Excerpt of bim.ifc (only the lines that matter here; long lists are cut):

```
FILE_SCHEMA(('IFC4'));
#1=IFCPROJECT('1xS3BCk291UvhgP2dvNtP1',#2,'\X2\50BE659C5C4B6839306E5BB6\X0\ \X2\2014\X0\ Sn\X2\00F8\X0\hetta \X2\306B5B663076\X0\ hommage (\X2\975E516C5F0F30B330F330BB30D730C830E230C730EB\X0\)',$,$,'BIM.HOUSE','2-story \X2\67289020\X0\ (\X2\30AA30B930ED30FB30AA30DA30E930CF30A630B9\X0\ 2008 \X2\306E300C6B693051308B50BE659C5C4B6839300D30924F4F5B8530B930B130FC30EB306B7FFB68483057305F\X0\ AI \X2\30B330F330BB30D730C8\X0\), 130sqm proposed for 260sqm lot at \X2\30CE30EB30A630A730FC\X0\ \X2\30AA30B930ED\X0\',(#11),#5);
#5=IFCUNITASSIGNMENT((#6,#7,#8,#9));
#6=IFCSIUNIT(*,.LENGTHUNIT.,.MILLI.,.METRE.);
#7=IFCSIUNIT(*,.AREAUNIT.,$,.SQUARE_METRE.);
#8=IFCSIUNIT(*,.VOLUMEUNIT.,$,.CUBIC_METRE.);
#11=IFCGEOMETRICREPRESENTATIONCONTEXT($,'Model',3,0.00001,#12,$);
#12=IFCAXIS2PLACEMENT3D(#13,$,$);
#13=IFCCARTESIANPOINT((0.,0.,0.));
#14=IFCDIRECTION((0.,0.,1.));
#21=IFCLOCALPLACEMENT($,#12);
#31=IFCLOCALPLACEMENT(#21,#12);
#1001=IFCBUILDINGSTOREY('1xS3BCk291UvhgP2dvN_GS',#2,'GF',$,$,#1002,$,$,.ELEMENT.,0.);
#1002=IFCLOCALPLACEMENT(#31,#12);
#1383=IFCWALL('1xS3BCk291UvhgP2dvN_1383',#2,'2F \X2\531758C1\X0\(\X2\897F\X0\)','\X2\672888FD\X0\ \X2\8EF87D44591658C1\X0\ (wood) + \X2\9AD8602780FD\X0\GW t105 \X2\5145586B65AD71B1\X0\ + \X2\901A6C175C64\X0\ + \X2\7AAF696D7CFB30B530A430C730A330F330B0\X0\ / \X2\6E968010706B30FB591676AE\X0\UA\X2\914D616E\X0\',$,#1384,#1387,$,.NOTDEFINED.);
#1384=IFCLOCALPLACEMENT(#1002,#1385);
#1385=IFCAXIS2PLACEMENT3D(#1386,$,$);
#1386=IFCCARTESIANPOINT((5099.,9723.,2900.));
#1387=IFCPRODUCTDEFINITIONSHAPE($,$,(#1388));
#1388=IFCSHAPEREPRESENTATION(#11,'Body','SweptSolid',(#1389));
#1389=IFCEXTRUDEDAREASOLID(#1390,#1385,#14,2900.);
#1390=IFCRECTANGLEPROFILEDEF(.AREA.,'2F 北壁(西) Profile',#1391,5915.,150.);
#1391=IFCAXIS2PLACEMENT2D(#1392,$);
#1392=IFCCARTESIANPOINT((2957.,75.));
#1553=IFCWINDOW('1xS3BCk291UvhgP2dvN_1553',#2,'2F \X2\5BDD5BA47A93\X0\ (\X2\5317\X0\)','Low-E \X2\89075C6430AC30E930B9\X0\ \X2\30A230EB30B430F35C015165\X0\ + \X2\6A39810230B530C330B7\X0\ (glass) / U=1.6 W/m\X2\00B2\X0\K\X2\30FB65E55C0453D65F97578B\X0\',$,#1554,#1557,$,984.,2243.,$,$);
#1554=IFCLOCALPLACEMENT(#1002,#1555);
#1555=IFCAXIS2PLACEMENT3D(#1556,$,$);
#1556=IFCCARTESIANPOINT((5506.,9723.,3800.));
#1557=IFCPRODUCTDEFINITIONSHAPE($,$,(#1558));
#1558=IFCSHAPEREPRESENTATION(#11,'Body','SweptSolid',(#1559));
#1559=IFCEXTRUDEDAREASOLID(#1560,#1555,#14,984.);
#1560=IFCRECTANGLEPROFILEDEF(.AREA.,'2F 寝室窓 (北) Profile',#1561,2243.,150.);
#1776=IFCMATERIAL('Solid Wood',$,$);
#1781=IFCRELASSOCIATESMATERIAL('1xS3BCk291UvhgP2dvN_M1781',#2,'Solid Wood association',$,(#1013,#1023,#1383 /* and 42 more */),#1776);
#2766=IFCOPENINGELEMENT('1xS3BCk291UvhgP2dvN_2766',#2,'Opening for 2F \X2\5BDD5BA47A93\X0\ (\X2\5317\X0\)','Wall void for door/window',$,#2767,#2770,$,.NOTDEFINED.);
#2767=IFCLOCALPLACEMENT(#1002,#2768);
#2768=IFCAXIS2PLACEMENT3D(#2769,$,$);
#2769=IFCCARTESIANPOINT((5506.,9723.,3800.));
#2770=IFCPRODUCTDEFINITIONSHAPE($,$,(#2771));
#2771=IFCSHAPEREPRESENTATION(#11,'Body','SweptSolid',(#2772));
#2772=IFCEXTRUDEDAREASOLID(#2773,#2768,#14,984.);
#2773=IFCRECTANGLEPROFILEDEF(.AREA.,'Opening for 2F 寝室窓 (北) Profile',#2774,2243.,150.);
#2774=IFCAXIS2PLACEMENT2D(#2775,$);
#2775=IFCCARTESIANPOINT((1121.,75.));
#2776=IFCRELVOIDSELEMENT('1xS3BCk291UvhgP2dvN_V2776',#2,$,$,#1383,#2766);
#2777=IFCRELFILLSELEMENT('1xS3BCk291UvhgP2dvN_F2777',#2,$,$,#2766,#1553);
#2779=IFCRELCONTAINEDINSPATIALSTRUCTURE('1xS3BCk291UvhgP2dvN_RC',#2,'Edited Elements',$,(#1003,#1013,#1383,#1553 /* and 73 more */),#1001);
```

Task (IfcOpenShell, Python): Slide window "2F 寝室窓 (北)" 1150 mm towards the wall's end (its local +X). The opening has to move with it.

```python
import ifcopenshell
import ifcopenshell.api.geometry
import ifcopenshell.util.placement

model = ifcopenshell.open("bim.ifc")

window = model.by_id(1553)
opening = window.FillsVoids[0].RelatingOpeningElement
wall = opening.VoidsElements[0].RelatingBuildingElement

wall_matrix = ifcopenshell.util.placement.get_local_placement(wall.ObjectPlacement)
shift = wall_matrix[:3, 0] * 1150.0
before = ifcopenshell.util.placement.get_local_placement(window.ObjectPlacement)[:3, 3].copy()

# The window is not placed relative to its opening, so move both.
for product in (opening, window):
    matrix = ifcopenshell.util.placement.get_local_placement(product.ObjectPlacement)
    matrix[:3, 3] += shift
    ifcopenshell.api.geometry.edit_object_placement(model, product=product, matrix=matrix, is_si=False)

after = ifcopenshell.util.placement.get_local_placement(window.ObjectPlacement)[:3, 3]
print("window moved by", (after - before).round(3) + 0.0)

model.write("bim_v2.ifc")
```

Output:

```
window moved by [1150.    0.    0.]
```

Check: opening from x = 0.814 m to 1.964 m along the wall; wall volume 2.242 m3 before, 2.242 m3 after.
